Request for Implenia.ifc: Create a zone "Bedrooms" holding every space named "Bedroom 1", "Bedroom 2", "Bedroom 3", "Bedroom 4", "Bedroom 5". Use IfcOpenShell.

First a look at what the model holds.

```python
import ifcopenshell

model = ifcopenshell.open("Implenia.ifc")
print(model.schema)
seen = {}
for space in model.by_type("IfcSpace"):
    seen[space.LongName] = seen.get(space.LongName, 0) + 1
for name, count in sorted(seen.items(), key=str):
    print(count, "x", name)
print("zones:", [z.Name for z in model.by_type("IfcZone")][:20])
```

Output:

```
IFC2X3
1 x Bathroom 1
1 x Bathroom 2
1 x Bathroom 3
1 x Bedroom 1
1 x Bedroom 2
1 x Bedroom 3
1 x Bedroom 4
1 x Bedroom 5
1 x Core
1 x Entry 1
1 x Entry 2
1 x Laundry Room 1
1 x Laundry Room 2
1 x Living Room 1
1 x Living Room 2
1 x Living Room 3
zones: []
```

```python
import ifcopenshell
import ifcopenshell.api.group
import ifcopenshell.api.root

model = ifcopenshell.open("Implenia.ifc")

names = {"Bedroom 1", "Bedroom 2", "Bedroom 3", "Bedroom 4", "Bedroom 5"}
spaces = [s for s in model.by_type("IfcSpace") if s.LongName in names]

zone = ifcopenshell.api.root.create_entity(model, ifc_class="IfcZone", name="Bedrooms")
ifcopenshell.api.group.assign_group(model, products=spaces, group=zone)
print(len(spaces), "spaces in", zone.Name)

model.write("Implenia_rev.ifc")
```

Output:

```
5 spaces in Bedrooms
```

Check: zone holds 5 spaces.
